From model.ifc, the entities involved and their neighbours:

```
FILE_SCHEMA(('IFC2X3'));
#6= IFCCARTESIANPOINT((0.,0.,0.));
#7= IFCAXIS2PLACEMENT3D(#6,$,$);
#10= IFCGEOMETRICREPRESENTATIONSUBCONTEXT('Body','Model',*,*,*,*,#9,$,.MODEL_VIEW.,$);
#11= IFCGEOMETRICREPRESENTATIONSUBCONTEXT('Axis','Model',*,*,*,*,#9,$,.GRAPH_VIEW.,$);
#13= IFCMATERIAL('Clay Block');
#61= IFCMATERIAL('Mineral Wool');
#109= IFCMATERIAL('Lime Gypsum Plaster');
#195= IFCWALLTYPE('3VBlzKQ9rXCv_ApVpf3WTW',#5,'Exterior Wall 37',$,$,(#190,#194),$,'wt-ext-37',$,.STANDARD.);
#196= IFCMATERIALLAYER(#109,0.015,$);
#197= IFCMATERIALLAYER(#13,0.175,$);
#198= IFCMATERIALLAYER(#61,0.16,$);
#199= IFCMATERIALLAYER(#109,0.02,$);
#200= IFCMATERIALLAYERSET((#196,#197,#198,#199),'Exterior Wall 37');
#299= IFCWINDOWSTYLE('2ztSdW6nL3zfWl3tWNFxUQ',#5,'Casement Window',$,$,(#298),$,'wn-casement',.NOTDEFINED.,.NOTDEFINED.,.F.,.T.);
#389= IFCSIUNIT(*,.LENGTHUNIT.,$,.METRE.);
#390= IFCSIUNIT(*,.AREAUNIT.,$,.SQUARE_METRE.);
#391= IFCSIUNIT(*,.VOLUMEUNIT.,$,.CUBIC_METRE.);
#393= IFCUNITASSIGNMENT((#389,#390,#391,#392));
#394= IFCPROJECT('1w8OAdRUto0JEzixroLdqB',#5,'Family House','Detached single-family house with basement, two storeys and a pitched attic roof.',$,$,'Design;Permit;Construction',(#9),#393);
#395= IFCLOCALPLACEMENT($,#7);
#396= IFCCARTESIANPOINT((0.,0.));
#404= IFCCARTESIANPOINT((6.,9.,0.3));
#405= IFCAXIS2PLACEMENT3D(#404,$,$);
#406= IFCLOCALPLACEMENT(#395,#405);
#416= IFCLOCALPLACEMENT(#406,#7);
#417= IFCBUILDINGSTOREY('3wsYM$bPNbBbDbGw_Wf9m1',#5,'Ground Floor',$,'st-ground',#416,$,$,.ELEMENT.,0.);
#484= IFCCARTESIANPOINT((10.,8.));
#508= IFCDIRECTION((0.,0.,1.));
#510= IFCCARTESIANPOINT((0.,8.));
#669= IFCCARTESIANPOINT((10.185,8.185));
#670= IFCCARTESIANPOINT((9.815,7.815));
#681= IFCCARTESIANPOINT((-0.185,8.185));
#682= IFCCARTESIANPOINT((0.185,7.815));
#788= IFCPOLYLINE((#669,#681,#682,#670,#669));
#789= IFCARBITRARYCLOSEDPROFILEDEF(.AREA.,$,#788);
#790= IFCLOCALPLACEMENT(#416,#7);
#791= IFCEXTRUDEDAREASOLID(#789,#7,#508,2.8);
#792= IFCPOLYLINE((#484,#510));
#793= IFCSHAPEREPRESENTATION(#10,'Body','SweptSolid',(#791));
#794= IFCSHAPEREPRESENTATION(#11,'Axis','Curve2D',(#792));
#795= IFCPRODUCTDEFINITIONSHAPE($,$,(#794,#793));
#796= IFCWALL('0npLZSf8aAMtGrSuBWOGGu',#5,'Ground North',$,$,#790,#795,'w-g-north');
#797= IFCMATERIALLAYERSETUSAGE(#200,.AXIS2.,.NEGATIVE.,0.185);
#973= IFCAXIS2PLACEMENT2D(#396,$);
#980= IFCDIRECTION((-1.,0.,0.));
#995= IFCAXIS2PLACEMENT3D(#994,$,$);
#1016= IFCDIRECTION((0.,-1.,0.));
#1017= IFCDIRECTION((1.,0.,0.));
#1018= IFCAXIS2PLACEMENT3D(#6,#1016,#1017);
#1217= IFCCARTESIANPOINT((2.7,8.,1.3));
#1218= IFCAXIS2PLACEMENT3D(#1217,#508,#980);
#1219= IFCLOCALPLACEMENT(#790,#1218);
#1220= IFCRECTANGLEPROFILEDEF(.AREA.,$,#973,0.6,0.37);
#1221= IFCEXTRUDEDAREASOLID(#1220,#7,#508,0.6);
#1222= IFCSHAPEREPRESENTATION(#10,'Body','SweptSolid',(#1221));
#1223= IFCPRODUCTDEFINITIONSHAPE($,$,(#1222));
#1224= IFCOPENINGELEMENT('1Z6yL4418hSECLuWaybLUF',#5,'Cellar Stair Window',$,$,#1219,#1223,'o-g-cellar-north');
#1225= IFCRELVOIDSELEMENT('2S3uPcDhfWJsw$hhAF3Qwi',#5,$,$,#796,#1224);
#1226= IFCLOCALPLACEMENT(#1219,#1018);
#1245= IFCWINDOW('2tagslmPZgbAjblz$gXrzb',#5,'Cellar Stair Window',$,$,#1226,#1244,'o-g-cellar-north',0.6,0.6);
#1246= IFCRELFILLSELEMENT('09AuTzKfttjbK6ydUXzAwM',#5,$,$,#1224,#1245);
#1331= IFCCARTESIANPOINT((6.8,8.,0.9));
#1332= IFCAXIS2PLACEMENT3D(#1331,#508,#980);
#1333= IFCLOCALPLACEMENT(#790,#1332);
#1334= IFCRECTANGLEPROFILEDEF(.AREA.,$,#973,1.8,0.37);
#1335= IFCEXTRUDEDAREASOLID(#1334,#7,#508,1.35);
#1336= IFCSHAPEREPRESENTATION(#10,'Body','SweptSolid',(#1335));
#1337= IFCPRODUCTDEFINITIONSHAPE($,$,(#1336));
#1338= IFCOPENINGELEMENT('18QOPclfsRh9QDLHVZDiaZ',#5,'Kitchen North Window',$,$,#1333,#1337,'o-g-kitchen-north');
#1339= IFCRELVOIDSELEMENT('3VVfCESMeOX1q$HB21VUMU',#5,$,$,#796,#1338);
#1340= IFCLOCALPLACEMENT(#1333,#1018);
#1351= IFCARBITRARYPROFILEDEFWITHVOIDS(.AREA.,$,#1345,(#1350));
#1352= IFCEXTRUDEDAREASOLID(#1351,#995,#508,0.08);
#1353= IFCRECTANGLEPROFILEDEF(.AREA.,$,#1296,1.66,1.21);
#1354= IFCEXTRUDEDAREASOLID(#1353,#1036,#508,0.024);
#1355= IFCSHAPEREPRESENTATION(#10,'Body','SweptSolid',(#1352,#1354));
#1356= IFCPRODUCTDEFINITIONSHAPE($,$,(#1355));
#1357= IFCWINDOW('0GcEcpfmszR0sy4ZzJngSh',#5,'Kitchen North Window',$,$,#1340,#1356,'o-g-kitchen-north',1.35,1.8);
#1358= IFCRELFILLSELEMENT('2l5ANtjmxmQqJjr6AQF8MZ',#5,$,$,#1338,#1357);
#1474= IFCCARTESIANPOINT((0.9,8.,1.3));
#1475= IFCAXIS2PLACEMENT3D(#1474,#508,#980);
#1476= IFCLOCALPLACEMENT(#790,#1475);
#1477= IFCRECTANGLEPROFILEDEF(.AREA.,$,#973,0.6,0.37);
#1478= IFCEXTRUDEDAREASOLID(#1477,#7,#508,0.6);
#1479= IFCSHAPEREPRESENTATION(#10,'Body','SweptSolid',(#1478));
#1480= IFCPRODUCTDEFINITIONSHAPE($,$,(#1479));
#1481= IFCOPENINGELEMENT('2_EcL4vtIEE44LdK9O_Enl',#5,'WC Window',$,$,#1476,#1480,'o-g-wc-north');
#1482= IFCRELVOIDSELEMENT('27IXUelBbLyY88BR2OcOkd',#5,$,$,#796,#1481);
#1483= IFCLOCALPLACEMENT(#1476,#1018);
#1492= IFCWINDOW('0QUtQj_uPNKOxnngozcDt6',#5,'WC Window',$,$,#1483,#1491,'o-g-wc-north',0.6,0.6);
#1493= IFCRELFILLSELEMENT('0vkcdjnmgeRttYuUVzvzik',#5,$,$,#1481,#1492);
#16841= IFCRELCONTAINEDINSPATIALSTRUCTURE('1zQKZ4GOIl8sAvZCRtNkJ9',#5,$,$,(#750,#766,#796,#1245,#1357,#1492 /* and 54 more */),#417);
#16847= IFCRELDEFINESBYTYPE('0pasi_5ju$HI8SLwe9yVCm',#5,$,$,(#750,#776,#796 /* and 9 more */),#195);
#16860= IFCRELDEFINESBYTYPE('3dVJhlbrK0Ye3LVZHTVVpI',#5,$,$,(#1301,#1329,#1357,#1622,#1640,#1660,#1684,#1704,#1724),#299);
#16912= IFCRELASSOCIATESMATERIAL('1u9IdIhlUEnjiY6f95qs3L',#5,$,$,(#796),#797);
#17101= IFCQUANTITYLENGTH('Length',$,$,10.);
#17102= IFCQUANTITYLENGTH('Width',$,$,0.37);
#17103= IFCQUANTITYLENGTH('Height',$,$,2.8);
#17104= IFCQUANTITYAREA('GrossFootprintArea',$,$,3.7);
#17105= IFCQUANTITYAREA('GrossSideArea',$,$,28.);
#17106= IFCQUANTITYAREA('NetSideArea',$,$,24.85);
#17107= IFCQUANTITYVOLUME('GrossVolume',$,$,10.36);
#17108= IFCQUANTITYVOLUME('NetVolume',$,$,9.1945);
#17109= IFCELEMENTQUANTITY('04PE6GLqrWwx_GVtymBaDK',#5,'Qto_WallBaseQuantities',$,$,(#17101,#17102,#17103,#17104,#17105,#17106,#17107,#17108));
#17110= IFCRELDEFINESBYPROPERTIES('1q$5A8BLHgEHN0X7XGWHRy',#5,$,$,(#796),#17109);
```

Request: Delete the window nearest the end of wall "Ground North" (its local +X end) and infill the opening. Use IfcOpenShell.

```python
import ifcopenshell
import ifcopenshell.api.feature
import ifcopenshell.api.pset
import ifcopenshell.api.root
import ifcopenshell.geom
import ifcopenshell.util.element
import ifcopenshell.util.shape
import ifcopenshell.util.unit

model = ifcopenshell.open("model.ifc")
area_scale = ifcopenshell.util.unit.calculate_unit_scale(model, "AREAUNIT")
volume_scale = ifcopenshell.util.unit.calculate_unit_scale(model, "VOLUMEUNIT")
settings = ifcopenshell.geom.settings()


def volume(element):
    """Net volume in cubic metres, openings subtracted."""
    shape = ifcopenshell.geom.create_shape(settings, element)
    return ifcopenshell.util.shape.get_volume(shape.geometry)


window = model.by_guid("0GcEcpfmszR0sy4ZzJngSh")
opening = window.FillsVoids[0].RelatingOpeningElement
wall = opening.VoidsElements[0].RelatingBuildingElement
before = volume(wall)

ifcopenshell.api.root.remove_product(model, product=window)
ifcopenshell.api.feature.remove_feature(model, feature=opening)

after = volume(wall)
thickness = 0.37  # wall thickness in metres

# Update the wall's stored quantities.
qto = model.by_id(ifcopenshell.util.element.get_pset(wall, "Qto_WallBaseQuantities", should_inherit=False)["id"])
ifcopenshell.api.pset.edit_qto(model, qto=qto, properties={
    "NetSideArea": after / thickness / area_scale,
    "NetVolume": after / volume_scale,
})

print(f"wall volume {before:.3f} -> {after:.3f} m3")

model.write("model_v2.ifc")
```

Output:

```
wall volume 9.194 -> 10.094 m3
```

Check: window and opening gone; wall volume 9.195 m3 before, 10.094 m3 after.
